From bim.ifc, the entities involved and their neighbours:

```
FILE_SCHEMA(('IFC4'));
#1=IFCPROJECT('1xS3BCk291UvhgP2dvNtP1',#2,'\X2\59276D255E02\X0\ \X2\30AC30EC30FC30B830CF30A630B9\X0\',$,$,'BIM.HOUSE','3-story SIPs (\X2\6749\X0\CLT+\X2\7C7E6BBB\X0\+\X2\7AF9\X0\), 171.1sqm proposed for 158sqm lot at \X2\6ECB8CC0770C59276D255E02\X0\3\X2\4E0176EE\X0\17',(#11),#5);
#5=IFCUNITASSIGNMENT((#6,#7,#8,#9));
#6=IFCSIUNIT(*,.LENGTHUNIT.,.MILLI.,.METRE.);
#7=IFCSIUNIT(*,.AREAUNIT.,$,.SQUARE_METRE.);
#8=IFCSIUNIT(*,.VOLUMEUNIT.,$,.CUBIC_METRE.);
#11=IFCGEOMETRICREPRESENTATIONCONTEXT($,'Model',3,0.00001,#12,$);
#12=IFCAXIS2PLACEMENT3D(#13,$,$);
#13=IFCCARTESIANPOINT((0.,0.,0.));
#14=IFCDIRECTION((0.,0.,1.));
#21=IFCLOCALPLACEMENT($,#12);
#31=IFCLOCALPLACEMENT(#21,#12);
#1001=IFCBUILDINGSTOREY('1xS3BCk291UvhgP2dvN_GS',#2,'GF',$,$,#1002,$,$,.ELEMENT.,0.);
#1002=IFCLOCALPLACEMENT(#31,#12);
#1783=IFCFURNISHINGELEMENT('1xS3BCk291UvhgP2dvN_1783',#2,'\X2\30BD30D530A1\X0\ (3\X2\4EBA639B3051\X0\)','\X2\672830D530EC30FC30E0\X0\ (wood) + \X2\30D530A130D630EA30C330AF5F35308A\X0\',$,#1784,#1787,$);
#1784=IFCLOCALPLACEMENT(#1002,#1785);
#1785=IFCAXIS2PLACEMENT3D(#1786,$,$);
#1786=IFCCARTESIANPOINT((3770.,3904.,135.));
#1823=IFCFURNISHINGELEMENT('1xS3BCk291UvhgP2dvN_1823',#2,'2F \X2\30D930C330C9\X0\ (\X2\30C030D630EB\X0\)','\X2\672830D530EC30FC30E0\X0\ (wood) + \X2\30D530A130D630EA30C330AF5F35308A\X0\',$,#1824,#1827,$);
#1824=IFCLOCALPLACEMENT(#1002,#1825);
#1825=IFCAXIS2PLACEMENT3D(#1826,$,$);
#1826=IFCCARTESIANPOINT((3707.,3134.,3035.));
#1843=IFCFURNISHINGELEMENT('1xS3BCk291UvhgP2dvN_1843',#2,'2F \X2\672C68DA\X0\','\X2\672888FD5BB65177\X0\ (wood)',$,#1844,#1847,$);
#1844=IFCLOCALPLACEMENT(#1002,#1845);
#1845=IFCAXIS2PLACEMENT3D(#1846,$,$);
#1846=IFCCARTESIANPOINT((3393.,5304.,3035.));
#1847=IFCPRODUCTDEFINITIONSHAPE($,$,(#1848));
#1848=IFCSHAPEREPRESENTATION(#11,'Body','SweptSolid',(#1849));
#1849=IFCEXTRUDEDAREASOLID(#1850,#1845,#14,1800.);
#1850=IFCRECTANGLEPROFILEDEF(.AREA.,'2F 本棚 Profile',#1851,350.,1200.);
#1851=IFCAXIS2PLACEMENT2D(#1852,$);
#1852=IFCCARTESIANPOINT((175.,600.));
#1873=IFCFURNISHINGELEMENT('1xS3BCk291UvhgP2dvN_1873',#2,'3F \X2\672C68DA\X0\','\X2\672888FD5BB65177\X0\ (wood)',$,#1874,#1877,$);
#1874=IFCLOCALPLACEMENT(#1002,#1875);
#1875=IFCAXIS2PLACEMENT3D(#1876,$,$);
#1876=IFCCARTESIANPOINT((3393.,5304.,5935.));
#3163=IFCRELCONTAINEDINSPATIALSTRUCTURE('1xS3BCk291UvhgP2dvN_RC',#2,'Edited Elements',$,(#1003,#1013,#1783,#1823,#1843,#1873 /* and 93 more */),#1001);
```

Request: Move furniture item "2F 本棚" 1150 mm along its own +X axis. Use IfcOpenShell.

```python
import ifcopenshell
import ifcopenshell.api.geometry
import ifcopenshell.util.placement

model = ifcopenshell.open("bim.ifc")

item = model.by_guid("1xS3BCk291UvhgP2dvN_1843")
matrix = ifcopenshell.util.placement.get_local_placement(item.ObjectPlacement)
matrix[:3, 3] += matrix[:3, 0] * 1150.0
ifcopenshell.api.geometry.edit_object_placement(model, product=item, matrix=matrix, is_si=False)

print(ifcopenshell.util.placement.get_local_placement(item.ObjectPlacement).round(3) + 0.0)

model.write("bim_edited.ifc")
```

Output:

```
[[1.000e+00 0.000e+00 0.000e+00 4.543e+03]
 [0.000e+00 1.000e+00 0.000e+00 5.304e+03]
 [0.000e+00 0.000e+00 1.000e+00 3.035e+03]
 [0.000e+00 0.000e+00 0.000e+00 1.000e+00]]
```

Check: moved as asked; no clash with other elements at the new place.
